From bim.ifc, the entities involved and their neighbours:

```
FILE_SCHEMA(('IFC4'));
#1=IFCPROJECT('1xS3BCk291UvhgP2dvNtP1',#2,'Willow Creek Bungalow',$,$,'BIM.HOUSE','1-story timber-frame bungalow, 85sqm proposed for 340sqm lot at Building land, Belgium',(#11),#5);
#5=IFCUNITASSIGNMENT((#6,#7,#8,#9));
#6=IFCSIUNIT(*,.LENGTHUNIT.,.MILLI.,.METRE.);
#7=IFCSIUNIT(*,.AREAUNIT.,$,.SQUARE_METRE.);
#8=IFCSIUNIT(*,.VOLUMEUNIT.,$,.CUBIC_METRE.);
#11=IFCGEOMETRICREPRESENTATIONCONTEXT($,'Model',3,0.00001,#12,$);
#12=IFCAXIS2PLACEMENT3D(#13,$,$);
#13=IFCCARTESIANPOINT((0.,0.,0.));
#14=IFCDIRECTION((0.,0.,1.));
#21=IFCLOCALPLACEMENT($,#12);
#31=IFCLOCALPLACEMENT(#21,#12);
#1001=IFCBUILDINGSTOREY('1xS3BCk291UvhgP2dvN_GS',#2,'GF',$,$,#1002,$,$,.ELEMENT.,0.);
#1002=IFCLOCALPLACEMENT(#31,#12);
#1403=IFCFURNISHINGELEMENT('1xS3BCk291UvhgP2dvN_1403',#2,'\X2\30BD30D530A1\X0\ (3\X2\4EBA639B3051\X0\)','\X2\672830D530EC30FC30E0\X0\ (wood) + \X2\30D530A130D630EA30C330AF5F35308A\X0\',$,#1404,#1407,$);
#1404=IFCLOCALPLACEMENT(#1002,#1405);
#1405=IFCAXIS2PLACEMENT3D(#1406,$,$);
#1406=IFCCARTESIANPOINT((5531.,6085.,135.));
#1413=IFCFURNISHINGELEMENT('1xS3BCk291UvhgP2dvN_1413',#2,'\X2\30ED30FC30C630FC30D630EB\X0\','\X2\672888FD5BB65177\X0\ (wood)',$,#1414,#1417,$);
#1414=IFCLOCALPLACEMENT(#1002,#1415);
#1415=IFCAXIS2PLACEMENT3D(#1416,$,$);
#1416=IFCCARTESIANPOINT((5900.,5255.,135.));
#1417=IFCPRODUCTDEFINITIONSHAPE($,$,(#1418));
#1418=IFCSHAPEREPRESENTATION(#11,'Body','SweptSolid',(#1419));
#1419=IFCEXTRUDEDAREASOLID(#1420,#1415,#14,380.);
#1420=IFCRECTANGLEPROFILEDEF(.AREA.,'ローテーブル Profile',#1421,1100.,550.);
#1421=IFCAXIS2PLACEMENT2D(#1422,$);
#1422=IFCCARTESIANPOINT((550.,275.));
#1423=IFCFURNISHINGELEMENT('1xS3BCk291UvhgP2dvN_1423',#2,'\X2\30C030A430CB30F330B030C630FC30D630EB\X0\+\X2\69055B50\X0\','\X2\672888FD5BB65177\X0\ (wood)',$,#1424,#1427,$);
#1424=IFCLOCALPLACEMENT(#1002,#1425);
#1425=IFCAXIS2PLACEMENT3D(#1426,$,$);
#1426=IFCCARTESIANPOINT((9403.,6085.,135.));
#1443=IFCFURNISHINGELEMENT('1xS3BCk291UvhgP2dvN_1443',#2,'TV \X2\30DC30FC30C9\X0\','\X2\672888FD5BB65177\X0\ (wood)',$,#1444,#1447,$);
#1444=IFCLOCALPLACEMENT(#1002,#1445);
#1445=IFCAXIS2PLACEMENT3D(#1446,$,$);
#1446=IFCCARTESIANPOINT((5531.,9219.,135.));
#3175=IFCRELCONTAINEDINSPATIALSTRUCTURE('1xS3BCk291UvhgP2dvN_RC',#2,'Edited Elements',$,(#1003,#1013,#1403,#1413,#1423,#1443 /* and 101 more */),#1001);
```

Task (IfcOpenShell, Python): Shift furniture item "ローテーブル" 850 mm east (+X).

```python
import ifcopenshell
import ifcopenshell.api.geometry
import ifcopenshell.util.placement
import ifcopenshell.util.unit

model = ifcopenshell.open("bim.ifc")
unit_scale = ifcopenshell.util.unit.calculate_unit_scale(model)

item = model.by_guid("1xS3BCk291UvhgP2dvN_1413")
matrix = ifcopenshell.util.placement.get_local_placement(item.ObjectPlacement)
matrix[0, 3] += 0.85 / unit_scale
ifcopenshell.api.geometry.edit_object_placement(model, product=item, matrix=matrix, is_si=False)

print(ifcopenshell.util.placement.get_local_placement(item.ObjectPlacement).round(3) + 0.0)

model.write("bim-out.ifc")
```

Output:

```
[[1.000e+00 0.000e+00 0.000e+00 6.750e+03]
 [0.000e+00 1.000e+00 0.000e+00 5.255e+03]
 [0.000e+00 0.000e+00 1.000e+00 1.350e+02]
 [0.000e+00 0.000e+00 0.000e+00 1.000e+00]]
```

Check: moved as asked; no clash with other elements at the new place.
